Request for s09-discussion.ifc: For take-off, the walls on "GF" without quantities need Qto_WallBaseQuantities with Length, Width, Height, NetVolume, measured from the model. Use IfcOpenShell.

First a look at what the model holds.

```python
import ifcopenshell
import ifcopenshell.util.element
import ifcopenshell.util.unit

model = ifcopenshell.open("s09-discussion.ifc")
print(model.schema)
for unit_type in ("LENGTHUNIT", "AREAUNIT", "VOLUMEUNIT"):
    print(unit_type, ifcopenshell.util.unit.calculate_unit_scale(model, unit_type))
storey = next(s for s in model.by_type("IfcBuildingStorey") if s.Name == "GF")
walls = [e for e in ifcopenshell.util.element.get_decomposition(storey) if e.is_a("IfcWall")]
for e in sorted(walls, key=lambda e: e.id()):
    print(e.id(), e.is_a(), e.Name, list(ifcopenshell.util.element.get_psets(e, qtos_only=True)), sep=" | ")
```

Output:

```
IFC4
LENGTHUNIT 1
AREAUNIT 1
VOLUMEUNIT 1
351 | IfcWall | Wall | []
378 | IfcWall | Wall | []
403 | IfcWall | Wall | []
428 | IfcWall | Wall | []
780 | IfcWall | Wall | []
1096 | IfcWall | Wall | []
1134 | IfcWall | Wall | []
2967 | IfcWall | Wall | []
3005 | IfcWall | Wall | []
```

```python
import ifcopenshell
import ifcopenshell.api.pset
import ifcopenshell.geom
import ifcopenshell.util.element
import ifcopenshell.util.shape
import ifcopenshell.util.unit

model = ifcopenshell.open("s09-discussion.ifc")
unit_scale = ifcopenshell.util.unit.calculate_unit_scale(model)
volume_scale = ifcopenshell.util.unit.calculate_unit_scale(model, "VOLUMEUNIT")
settings = ifcopenshell.geom.settings()

storey = next(s for s in model.by_type("IfcBuildingStorey") if s.Name == "GF")
walls = [e for e in ifcopenshell.util.element.get_decomposition(storey) if e.is_a("IfcWall")]

for e in sorted(walls, key=lambda e: e.id()):
    if ifcopenshell.util.element.get_psets(e, qtos_only=True, should_inherit=False):
        continue
    # Geometry comes back in metres, in the element's own axes.
    shape = ifcopenshell.geom.create_shape(settings, e)
    values = {
        "Length": ifcopenshell.util.shape.get_x(shape.geometry) / unit_scale,
        "Width": ifcopenshell.util.shape.get_y(shape.geometry) / unit_scale,
        "Height": ifcopenshell.util.shape.get_z(shape.geometry) / unit_scale,
        "NetVolume": ifcopenshell.util.shape.get_volume(shape.geometry) / volume_scale,
    }
    qto = ifcopenshell.api.pset.add_qto(model, product=e, name="Qto_WallBaseQuantities")
    ifcopenshell.api.pset.edit_qto(model, qto=qto, properties=values)
    print(e.id(), {k: round(v, 3) for k, v in values.items()})

model.write("s09-discussion-out.ifc")
```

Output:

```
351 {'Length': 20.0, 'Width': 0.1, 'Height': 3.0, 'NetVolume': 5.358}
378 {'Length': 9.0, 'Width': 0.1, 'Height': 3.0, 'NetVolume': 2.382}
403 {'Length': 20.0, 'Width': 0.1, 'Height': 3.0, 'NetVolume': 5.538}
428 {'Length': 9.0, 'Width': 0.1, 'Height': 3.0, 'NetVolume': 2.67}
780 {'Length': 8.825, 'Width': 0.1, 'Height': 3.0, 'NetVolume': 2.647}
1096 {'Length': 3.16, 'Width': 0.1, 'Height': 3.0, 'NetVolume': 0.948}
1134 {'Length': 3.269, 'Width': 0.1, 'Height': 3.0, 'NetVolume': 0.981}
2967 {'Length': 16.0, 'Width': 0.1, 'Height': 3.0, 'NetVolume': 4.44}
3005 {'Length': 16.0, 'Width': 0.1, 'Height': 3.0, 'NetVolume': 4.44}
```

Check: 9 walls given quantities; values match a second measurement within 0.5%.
